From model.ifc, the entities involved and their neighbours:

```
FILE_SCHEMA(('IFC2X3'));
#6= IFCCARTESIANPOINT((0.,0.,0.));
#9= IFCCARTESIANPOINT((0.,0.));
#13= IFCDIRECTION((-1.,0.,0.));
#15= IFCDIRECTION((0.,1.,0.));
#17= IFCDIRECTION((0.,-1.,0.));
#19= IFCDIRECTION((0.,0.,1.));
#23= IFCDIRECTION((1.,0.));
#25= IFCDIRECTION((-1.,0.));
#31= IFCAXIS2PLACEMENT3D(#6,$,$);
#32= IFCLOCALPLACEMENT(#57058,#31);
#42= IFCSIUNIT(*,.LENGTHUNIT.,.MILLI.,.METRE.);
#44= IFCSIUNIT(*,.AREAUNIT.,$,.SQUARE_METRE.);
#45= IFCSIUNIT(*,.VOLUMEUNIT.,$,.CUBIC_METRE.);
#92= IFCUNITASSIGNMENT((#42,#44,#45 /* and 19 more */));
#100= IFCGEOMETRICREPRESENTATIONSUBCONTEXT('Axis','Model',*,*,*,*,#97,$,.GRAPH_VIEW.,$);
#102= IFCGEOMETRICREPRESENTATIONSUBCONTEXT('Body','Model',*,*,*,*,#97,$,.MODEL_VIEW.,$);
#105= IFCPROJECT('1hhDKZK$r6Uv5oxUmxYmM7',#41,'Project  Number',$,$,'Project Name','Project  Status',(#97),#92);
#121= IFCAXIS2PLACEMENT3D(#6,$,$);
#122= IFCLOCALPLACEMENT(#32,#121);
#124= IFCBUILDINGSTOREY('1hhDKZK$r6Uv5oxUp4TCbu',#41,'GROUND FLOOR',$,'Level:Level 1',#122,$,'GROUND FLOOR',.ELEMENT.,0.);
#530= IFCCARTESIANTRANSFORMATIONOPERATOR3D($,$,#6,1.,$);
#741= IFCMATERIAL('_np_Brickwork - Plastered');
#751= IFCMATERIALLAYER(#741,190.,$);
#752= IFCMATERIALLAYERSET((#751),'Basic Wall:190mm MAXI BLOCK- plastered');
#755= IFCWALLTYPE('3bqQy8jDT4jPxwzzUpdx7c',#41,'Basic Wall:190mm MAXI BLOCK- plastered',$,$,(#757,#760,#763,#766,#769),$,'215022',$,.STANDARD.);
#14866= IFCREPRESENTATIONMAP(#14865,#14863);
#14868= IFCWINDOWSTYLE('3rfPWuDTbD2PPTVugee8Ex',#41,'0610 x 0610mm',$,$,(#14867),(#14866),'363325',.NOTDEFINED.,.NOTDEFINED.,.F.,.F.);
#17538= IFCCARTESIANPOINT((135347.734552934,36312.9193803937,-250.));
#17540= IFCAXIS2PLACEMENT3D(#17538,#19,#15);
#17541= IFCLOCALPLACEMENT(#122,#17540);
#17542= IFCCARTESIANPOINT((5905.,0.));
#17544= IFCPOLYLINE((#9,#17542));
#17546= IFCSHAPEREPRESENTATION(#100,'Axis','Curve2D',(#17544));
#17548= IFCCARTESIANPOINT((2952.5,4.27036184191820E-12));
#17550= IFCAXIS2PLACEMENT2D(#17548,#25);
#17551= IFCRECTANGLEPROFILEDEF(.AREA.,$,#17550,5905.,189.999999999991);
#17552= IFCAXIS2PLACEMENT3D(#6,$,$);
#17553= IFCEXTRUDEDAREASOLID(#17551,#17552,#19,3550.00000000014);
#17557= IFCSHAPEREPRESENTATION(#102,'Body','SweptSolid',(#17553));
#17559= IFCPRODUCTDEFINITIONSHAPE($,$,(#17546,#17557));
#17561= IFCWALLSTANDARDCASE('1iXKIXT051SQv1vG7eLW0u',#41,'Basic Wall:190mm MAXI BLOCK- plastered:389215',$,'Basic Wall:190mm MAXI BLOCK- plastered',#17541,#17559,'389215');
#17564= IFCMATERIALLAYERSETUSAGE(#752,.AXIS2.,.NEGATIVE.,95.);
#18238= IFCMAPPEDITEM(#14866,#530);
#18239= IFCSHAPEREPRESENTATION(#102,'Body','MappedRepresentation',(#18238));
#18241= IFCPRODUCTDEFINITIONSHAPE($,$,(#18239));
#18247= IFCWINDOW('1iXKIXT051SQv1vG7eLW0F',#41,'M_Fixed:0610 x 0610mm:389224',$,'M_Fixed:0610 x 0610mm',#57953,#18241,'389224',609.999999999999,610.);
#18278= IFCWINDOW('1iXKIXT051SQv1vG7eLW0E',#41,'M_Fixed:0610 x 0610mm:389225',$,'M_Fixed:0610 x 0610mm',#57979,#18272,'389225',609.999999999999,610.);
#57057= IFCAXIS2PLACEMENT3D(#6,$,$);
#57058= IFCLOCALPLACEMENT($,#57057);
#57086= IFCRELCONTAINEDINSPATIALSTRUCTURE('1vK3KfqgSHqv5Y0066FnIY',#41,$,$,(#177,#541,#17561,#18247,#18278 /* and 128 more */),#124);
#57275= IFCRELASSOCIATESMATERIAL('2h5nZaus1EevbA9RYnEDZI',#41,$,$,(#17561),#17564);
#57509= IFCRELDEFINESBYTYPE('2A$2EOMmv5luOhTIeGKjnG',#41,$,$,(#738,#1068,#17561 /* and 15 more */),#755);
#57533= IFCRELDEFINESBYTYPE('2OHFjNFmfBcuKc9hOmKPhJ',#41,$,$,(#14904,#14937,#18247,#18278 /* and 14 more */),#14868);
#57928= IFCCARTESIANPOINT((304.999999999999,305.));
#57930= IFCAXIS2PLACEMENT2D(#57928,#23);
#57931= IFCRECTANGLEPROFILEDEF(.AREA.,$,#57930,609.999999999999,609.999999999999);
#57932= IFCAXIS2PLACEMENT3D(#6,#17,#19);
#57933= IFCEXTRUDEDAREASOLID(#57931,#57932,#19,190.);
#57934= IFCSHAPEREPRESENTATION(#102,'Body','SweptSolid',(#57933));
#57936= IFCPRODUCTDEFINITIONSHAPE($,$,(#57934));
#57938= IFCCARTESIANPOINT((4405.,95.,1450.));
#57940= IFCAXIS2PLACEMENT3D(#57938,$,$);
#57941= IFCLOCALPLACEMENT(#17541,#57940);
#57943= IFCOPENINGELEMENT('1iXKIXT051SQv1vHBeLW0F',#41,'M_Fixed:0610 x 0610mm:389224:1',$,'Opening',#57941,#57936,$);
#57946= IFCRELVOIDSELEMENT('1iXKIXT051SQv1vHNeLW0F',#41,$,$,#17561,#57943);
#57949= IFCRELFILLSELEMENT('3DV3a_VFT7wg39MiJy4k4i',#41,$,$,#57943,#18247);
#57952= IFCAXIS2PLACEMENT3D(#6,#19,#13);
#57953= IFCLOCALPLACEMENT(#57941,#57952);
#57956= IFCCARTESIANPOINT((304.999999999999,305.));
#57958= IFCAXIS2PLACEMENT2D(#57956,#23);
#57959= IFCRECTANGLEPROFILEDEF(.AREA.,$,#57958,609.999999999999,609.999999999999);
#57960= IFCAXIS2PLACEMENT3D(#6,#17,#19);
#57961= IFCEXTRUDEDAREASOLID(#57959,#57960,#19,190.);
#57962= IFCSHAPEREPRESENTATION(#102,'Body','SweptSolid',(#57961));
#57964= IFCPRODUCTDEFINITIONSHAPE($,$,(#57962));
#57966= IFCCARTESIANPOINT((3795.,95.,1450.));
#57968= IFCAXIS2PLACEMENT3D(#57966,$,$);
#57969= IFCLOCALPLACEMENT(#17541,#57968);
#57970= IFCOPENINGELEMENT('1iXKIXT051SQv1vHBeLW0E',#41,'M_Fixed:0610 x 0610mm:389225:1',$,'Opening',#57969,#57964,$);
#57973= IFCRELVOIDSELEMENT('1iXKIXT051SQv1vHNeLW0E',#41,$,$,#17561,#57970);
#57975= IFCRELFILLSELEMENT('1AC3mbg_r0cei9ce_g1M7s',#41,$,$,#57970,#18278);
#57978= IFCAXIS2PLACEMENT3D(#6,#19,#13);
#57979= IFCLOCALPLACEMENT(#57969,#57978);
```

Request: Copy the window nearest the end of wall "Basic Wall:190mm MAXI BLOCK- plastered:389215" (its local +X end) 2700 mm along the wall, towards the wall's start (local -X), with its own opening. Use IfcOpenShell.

```python
import ifcopenshell
import ifcopenshell.api.feature
import ifcopenshell.api.geometry
import ifcopenshell.api.root
import ifcopenshell.geom
import ifcopenshell.util.element
import ifcopenshell.util.placement
import ifcopenshell.util.shape

model = ifcopenshell.open("model.ifc")
settings = ifcopenshell.geom.settings()


def volume(element):
    """Net volume in cubic metres, openings subtracted."""
    shape = ifcopenshell.geom.create_shape(settings, element)
    return ifcopenshell.util.shape.get_volume(shape.geometry)


def reuse_history(source, copy):
    """copy_class also copies each property set's owner history, people and application; keep the originals."""
    for rel in copy.IsDefinedBy:
        if rel.is_a("IfcRelDefinesByProperties") and (history := rel.RelatingPropertyDefinition.OwnerHistory):
            rel.RelatingPropertyDefinition.OwnerHistory = source.OwnerHistory
            ifcopenshell.util.element.remove_deep2(model, history)


window = model.by_guid("1iXKIXT051SQv1vG7eLW0F")
opening = window.FillsVoids[0].RelatingOpeningElement
wall = opening.VoidsElements[0].RelatingBuildingElement
before = volume(wall)
shift = ifcopenshell.util.placement.get_local_placement(wall.ObjectPlacement)[:3, 0] * -2700.0

# copy_class copies the void relationship, type, container and properties, but no geometry.
new_opening = ifcopenshell.api.root.copy_class(model, product=opening)
new_opening.Representation = ifcopenshell.util.element.copy_deep(
    model, opening.Representation, exclude=["IfcGeometricRepresentationContext", "IfcRepresentationMap"]
)
new_opening.Name = "M_Fixed:0610 x 0610mm"
new_window = ifcopenshell.api.root.copy_class(model, product=window)
new_window.Representation = ifcopenshell.util.element.copy_deep(
    model, window.Representation, exclude=["IfcGeometricRepresentationContext", "IfcRepresentationMap"]
)
new_window.Name = "M_Fixed:0610 x 0610mm"
new_window.Tag = None
reuse_history(window, new_window)
fills = ifcopenshell.api.feature.add_filling(model, opening=new_opening, element=new_window)
fills.OwnerHistory = new_window.OwnerHistory  # required in IFC2X3

for old, new in ((opening, new_opening), (window, new_window)):
    matrix = ifcopenshell.util.placement.get_local_placement(old.ObjectPlacement)
    matrix[:3, 3] += shift
    ifcopenshell.api.geometry.edit_object_placement(model, product=new, matrix=matrix, is_si=False)

after = volume(wall)

print(f"wall volume {before:.3f} -> {after:.3f} m3")

model.write("model_rev.ifc")
```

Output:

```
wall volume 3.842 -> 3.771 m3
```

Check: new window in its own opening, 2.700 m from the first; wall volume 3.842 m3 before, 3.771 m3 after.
